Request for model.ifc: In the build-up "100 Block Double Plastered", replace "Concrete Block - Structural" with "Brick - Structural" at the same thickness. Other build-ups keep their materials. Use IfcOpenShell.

First a look at what the model holds.

```python
import ifcopenshell
import ifcopenshell.util.element

model = ifcopenshell.open("model.ifc")
print(model.schema)
for layer_set in model.by_type("IfcMaterialLayerSet"):
    if layer_set.LayerSetName == "100 Block Double Plastered":
        for layer in layer_set.MaterialLayers:
            print(layer.id(), layer.Material and layer.Material.Name, layer.LayerThickness, sep=" | ")
        print(len(ifcopenshell.util.element.get_elements_by_material(model, layer_set)), "elements and types use it")
print(sorted(m.Name for m in model.by_type("IfcMaterial") if m.Name)[:60])
```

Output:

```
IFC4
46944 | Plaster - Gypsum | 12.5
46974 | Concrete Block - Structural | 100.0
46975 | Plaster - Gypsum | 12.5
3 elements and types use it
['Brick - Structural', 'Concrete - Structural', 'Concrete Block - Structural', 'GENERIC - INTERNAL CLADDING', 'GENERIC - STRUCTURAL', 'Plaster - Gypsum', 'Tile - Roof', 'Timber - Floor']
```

```python
import ifcopenshell
import ifcopenshell.api.material

model = ifcopenshell.open("model.ifc")

layer_set = next(s for s in model.by_type("IfcMaterialLayerSet") if s.LayerSetName == "100 Block Double Plastered")
layer = next(l for l in layer_set.MaterialLayers if l.Material and l.Material.Name == "Concrete Block - Structural")
material = next(m for m in model.by_type("IfcMaterial") if m.Name == "Brick - Structural")

# Point this one layer at the other material; renaming the old one would change it everywhere.
ifcopenshell.api.material.edit_layer(model, layer=layer, attributes={}, material=material)

print([l.Material.Name if l.Material else None for l in layer_set.MaterialLayers])

model.write("model_rev.ifc")
```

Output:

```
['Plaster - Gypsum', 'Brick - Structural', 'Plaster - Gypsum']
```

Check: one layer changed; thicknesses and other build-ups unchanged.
